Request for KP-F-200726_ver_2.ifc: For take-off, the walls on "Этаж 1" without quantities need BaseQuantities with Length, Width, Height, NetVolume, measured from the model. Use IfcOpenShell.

First a look at what the model holds.

```python
import ifcopenshell
import ifcopenshell.util.element
import ifcopenshell.util.unit

model = ifcopenshell.open("KP-F-200726_ver_2.ifc")
print(model.schema)
for unit_type in ("LENGTHUNIT", "AREAUNIT", "VOLUMEUNIT"):
    print(unit_type, ifcopenshell.util.unit.calculate_unit_scale(model, unit_type))
storey = next(s for s in model.by_type("IfcBuildingStorey") if s.Name == "Этаж 1")
walls = [e for e in ifcopenshell.util.element.get_decomposition(storey) if e.is_a("IfcWall")]
for e in sorted(walls, key=lambda e: e.id()):
    print(e.id(), e.is_a(), e.Name, list(ifcopenshell.util.element.get_psets(e, qtos_only=True)), sep=" | ")
```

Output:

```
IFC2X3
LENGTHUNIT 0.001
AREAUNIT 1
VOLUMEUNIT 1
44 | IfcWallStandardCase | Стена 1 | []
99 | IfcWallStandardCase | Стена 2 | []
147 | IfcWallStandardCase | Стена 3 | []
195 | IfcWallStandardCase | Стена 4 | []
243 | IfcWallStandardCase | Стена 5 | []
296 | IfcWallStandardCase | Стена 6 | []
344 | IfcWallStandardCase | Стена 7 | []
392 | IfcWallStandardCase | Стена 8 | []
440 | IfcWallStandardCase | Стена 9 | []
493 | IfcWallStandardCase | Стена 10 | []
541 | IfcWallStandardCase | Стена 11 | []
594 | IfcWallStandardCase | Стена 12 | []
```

```python
import ifcopenshell
import ifcopenshell.api.pset
import ifcopenshell.geom
import ifcopenshell.util.element
import ifcopenshell.util.shape
import ifcopenshell.util.unit

model = ifcopenshell.open("KP-F-200726_ver_2.ifc")
unit_scale = ifcopenshell.util.unit.calculate_unit_scale(model)
volume_scale = ifcopenshell.util.unit.calculate_unit_scale(model, "VOLUMEUNIT")
settings = ifcopenshell.geom.settings()

storey = next(s for s in model.by_type("IfcBuildingStorey") if s.Name == "Этаж 1")
walls = [e for e in ifcopenshell.util.element.get_decomposition(storey) if e.is_a("IfcWall")]

for e in sorted(walls, key=lambda e: e.id()):
    if ifcopenshell.util.element.get_psets(e, qtos_only=True, should_inherit=False):
        continue
    # Geometry comes back in metres, in the element's own axes.
    shape = ifcopenshell.geom.create_shape(settings, e)
    values = {
        "Length": ifcopenshell.util.shape.get_x(shape.geometry) / unit_scale,
        "Width": ifcopenshell.util.shape.get_y(shape.geometry) / unit_scale,
        "Height": ifcopenshell.util.shape.get_z(shape.geometry) / unit_scale,
        "NetVolume": ifcopenshell.util.shape.get_volume(shape.geometry) / volume_scale,
    }
    qto = ifcopenshell.api.pset.add_qto(model, product=e, name="BaseQuantities")
    ifcopenshell.api.pset.edit_qto(model, qto=qto, properties=values)
    print(e.id(), {k: round(v, 3) for k, v in values.items()})

model.write("KP-F-200726_ver_2_rev.ifc")
```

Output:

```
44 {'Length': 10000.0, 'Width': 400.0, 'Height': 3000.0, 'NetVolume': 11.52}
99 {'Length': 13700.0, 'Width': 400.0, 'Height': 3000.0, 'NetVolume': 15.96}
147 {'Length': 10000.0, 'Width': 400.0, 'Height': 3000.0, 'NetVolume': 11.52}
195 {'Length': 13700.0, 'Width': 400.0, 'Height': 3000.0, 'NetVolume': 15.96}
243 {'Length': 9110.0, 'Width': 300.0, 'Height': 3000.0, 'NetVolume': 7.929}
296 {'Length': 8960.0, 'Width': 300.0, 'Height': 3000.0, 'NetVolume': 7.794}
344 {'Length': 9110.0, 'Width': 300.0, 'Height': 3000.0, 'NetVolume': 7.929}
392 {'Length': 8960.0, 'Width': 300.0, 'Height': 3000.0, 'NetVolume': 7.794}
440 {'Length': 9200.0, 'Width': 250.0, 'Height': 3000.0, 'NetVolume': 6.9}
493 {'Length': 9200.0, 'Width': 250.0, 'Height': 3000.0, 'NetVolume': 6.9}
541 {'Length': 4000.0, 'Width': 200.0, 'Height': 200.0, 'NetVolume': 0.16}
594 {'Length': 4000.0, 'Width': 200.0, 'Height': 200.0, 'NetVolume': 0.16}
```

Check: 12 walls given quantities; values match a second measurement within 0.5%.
